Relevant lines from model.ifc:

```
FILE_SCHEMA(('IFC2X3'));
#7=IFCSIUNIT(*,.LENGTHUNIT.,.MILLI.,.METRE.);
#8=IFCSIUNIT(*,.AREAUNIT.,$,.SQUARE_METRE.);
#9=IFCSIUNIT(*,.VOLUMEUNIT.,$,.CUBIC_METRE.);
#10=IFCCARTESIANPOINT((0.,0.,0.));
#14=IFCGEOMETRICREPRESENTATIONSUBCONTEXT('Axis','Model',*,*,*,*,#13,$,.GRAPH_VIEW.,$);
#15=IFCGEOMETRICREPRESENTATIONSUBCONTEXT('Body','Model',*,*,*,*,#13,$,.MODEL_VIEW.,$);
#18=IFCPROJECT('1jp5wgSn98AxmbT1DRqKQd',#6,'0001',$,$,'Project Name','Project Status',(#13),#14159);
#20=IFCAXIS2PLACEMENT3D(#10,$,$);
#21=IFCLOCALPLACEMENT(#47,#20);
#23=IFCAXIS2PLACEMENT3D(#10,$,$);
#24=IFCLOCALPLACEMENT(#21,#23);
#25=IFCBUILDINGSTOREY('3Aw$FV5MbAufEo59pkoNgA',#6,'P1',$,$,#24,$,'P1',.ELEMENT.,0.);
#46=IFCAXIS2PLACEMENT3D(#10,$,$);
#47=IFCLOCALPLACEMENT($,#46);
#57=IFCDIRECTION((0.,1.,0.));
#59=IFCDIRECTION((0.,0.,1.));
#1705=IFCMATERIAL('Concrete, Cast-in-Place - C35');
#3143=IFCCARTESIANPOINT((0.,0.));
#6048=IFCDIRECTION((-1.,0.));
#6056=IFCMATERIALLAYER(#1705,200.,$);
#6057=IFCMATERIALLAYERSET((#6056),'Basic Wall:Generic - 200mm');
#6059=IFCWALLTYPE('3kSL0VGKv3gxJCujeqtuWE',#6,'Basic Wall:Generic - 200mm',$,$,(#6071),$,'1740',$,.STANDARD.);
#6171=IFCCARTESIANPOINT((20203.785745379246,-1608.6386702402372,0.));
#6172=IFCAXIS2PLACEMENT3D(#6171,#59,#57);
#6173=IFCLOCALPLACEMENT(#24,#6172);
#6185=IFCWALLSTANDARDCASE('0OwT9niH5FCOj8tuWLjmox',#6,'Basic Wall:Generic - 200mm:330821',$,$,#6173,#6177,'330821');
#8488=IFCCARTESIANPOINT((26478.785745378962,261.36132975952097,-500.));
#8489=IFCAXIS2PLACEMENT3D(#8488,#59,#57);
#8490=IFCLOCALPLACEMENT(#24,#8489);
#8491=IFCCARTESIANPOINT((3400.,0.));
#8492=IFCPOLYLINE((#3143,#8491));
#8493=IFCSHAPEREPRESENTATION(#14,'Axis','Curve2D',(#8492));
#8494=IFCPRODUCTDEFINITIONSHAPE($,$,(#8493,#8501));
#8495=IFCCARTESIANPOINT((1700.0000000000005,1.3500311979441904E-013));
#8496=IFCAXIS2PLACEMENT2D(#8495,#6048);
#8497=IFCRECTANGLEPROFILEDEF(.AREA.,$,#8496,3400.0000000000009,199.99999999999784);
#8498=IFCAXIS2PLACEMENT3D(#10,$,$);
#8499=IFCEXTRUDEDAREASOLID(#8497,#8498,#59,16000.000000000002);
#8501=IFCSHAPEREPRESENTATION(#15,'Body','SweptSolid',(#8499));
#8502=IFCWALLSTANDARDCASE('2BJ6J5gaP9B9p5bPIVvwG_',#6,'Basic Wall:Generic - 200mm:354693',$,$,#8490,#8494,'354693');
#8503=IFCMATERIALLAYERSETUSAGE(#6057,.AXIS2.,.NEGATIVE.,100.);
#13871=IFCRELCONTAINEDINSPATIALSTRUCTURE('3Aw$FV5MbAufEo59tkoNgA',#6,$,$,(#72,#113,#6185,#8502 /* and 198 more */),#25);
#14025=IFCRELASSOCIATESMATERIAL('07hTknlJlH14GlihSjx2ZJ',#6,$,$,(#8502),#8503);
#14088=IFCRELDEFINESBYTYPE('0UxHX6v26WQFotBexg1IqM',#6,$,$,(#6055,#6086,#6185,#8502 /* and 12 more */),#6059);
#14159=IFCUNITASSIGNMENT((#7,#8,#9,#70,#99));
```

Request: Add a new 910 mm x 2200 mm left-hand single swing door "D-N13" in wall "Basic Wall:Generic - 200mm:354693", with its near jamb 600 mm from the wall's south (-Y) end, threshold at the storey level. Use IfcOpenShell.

```python
import numpy as np
import ifcopenshell
import ifcopenshell.api.feature
import ifcopenshell.api.geometry
import ifcopenshell.api.root
import ifcopenshell.api.spatial
import ifcopenshell.api.type
import ifcopenshell.geom
import ifcopenshell.util.element
import ifcopenshell.util.placement
import ifcopenshell.util.representation
import ifcopenshell.util.shape
import ifcopenshell.util.unit

model = ifcopenshell.open("model.ifc")
unit_scale = ifcopenshell.util.unit.calculate_unit_scale(model)
settings = ifcopenshell.geom.settings()


def volume(element):
    """Net volume in cubic metres, openings subtracted."""
    shape = ifcopenshell.geom.create_shape(settings, element)
    return ifcopenshell.util.shape.get_volume(shape.geometry)


wall = model.by_guid("2BJ6J5gaP9B9p5bPIVvwG_")
storey = ifcopenshell.util.element.get_container(wall, ifc_class="IfcBuildingStorey")
context = ifcopenshell.util.representation.get_context(model, "Model", "Body", "MODEL_VIEW")
before = volume(wall)

width, height, from_end, sill = 0.91, 2.2, 0.6, 0.0  # metres

# The wall runs along its own X axis, and the end named is its -X end.
wall_shape = ifcopenshell.geom.create_shape(settings, wall)
x, y, z = ifcopenshell.util.shape.get_vertices(wall_shape.geometry).T
start = x.min() + from_end
face, thickness = float(y.min()), float(y.max() - y.min())
wall_matrix = ifcopenshell.util.placement.get_local_placement(wall.ObjectPlacement)
level = ifcopenshell.util.placement.get_local_placement(storey.ObjectPlacement)[2, 3]


def in_wall(x, y):
    """Placement at x, y metres in the wall's axes, at sill height."""
    matrix = wall_matrix.copy()
    matrix[:, 3] = wall_matrix @ np.array([x / unit_scale, y / unit_scale, 0.0, 1.0])
    matrix[2, 3] = level + sill / unit_scale
    return matrix


# Opening: a box that overshoots both wall faces by 50 mm.
opening = ifcopenshell.api.root.create_entity(model, ifc_class="IfcOpeningElement")
box = ifcopenshell.api.geometry.add_wall_representation(
    model, context=context, length=width, height=height, thickness=thickness + 0.1
)
ifcopenshell.api.geometry.assign_representation(model, product=opening, representation=box)
ifcopenshell.api.geometry.edit_object_placement(model, product=opening, matrix=in_wall(start, face - 0.05), is_si=False)
ifcopenshell.api.feature.add_feature(model, feature=opening, element=wall)

door = ifcopenshell.api.root.create_entity(model, ifc_class="IfcDoor", name="D-N13")
door.OverallWidth, door.OverallHeight = width / unit_scale, height / unit_scale
body = ifcopenshell.api.geometry.add_door_representation(
    model,
    context=context,
    overall_width=door.OverallWidth,
    overall_height=door.OverallHeight,
    operation_type="SINGLE_SWING_LEFT",
    lining_properties={"LiningDepth": thickness / unit_scale, "ThresholdDepth": thickness / unit_scale},
)
ifcopenshell.api.geometry.assign_representation(model, product=door, representation=body)
ifcopenshell.api.spatial.assign_container(model, products=[door], relating_structure=storey)
fills = ifcopenshell.api.feature.add_filling(model, opening=opening, element=door)
fills.OwnerHistory = door.OwnerHistory  # required in IFC2X3

# IFC2X3 keeps the operation on the door style.
style = ifcopenshell.api.root.create_entity(model, ifc_class="IfcDoorStyle", name="D-N13")
style.OperationType, style.ConstructionType = "SINGLE_SWING_LEFT", "NOTDEFINED"
style.ParameterTakesPrecedence = style.Sizeable = False
ifcopenshell.api.type.assign_type(model, related_objects=[door], relating_type=style)

# The lining spans the wall, so the door starts at the wall face.
ifcopenshell.api.geometry.edit_object_placement(model, product=door, matrix=in_wall(start, face), is_si=False)

after = volume(wall)

print(f"wall volume {before:.3f} -> {after:.3f} m3")

model.write("model-out.ifc")
```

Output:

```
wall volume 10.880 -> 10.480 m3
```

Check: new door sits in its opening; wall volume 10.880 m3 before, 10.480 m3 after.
